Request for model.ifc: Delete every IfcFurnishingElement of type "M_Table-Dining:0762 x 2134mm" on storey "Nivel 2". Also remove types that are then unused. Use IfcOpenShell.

First a look at what the model holds.

```python
import ifcopenshell
import ifcopenshell.util.element

model = ifcopenshell.open("model.ifc")
print(model.schema)
storey = next(s for s in model.by_type("IfcBuildingStorey") if s.Name == "Nivel 2")
furniture = [e for e in ifcopenshell.util.element.get_decomposition(storey) if e.is_a("IfcFurnishingElement")]
seen = {}
for e in furniture:
    element_type = ifcopenshell.util.element.get_type(e)
    name = element_type.Name if element_type not in (None, e) else None
    seen[name] = seen.get(name, 0) + 1
for name, count in sorted(seen.items(), key=str):
    print(count, "x", name)
```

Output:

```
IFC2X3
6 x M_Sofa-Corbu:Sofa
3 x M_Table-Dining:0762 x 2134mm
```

```python
import ifcopenshell
import ifcopenshell.api.root
import ifcopenshell.util.element

model = ifcopenshell.open("model.ifc")

storey = next(s for s in model.by_type("IfcBuildingStorey") if s.Name == "Nivel 2")
furniture = [e for e in ifcopenshell.util.element.get_decomposition(storey) if e.is_a("IfcFurnishingElement")]
targets = [e for e in furniture if (t := ifcopenshell.util.element.get_type(e)) not in (None, e) and t.Name == "M_Table-Dining:0762 x 2134mm"]
types = {ifcopenshell.util.element.get_type(e) for e in targets} - {None, *targets}

for e in targets:
    ifcopenshell.api.root.remove_product(model, product=e)
print(len(targets), "removed")

unused = [t for t in types if not ifcopenshell.util.element.get_types(t)]
for t in unused:
    ifcopenshell.api.root.remove_product(model, product=t)
print(len(unused), "unused types removed")

model.write("model-out.ifc")
```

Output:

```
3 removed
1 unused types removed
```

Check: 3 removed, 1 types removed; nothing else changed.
